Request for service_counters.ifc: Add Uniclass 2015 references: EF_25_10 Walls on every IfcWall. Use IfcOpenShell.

First a look at what the model holds.

```python
import ifcopenshell

model = ifcopenshell.open("service_counters.ifc")
print(model.schema)
print("classifications:", [c.Name for c in model.by_type("IfcClassification")])
for ifc_class in ("IfcDoor", "IfcRoof", "IfcStair", "IfcWall", "IfcWindow"):
    print(ifc_class, len(model.by_type(ifc_class)))
```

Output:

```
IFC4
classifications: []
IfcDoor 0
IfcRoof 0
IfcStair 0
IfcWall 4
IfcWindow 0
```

```python
import ifcopenshell
import ifcopenshell.api.classification

model = ifcopenshell.open("service_counters.ifc")

system = ifcopenshell.api.classification.add_classification(model, classification="Uniclass 2015")

codes = {
    "IfcWall": ("EF_25_10", "Walls"),
}
for ifc_class, (code, name) in codes.items():
    products = model.by_type(ifc_class)
    ifcopenshell.api.classification.add_reference(
        model, products=products, classification=system, identification=code, name=name
    )
    print(code, len(products))

model.write("service_counters_rev.ifc")
```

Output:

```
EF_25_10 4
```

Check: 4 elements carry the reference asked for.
